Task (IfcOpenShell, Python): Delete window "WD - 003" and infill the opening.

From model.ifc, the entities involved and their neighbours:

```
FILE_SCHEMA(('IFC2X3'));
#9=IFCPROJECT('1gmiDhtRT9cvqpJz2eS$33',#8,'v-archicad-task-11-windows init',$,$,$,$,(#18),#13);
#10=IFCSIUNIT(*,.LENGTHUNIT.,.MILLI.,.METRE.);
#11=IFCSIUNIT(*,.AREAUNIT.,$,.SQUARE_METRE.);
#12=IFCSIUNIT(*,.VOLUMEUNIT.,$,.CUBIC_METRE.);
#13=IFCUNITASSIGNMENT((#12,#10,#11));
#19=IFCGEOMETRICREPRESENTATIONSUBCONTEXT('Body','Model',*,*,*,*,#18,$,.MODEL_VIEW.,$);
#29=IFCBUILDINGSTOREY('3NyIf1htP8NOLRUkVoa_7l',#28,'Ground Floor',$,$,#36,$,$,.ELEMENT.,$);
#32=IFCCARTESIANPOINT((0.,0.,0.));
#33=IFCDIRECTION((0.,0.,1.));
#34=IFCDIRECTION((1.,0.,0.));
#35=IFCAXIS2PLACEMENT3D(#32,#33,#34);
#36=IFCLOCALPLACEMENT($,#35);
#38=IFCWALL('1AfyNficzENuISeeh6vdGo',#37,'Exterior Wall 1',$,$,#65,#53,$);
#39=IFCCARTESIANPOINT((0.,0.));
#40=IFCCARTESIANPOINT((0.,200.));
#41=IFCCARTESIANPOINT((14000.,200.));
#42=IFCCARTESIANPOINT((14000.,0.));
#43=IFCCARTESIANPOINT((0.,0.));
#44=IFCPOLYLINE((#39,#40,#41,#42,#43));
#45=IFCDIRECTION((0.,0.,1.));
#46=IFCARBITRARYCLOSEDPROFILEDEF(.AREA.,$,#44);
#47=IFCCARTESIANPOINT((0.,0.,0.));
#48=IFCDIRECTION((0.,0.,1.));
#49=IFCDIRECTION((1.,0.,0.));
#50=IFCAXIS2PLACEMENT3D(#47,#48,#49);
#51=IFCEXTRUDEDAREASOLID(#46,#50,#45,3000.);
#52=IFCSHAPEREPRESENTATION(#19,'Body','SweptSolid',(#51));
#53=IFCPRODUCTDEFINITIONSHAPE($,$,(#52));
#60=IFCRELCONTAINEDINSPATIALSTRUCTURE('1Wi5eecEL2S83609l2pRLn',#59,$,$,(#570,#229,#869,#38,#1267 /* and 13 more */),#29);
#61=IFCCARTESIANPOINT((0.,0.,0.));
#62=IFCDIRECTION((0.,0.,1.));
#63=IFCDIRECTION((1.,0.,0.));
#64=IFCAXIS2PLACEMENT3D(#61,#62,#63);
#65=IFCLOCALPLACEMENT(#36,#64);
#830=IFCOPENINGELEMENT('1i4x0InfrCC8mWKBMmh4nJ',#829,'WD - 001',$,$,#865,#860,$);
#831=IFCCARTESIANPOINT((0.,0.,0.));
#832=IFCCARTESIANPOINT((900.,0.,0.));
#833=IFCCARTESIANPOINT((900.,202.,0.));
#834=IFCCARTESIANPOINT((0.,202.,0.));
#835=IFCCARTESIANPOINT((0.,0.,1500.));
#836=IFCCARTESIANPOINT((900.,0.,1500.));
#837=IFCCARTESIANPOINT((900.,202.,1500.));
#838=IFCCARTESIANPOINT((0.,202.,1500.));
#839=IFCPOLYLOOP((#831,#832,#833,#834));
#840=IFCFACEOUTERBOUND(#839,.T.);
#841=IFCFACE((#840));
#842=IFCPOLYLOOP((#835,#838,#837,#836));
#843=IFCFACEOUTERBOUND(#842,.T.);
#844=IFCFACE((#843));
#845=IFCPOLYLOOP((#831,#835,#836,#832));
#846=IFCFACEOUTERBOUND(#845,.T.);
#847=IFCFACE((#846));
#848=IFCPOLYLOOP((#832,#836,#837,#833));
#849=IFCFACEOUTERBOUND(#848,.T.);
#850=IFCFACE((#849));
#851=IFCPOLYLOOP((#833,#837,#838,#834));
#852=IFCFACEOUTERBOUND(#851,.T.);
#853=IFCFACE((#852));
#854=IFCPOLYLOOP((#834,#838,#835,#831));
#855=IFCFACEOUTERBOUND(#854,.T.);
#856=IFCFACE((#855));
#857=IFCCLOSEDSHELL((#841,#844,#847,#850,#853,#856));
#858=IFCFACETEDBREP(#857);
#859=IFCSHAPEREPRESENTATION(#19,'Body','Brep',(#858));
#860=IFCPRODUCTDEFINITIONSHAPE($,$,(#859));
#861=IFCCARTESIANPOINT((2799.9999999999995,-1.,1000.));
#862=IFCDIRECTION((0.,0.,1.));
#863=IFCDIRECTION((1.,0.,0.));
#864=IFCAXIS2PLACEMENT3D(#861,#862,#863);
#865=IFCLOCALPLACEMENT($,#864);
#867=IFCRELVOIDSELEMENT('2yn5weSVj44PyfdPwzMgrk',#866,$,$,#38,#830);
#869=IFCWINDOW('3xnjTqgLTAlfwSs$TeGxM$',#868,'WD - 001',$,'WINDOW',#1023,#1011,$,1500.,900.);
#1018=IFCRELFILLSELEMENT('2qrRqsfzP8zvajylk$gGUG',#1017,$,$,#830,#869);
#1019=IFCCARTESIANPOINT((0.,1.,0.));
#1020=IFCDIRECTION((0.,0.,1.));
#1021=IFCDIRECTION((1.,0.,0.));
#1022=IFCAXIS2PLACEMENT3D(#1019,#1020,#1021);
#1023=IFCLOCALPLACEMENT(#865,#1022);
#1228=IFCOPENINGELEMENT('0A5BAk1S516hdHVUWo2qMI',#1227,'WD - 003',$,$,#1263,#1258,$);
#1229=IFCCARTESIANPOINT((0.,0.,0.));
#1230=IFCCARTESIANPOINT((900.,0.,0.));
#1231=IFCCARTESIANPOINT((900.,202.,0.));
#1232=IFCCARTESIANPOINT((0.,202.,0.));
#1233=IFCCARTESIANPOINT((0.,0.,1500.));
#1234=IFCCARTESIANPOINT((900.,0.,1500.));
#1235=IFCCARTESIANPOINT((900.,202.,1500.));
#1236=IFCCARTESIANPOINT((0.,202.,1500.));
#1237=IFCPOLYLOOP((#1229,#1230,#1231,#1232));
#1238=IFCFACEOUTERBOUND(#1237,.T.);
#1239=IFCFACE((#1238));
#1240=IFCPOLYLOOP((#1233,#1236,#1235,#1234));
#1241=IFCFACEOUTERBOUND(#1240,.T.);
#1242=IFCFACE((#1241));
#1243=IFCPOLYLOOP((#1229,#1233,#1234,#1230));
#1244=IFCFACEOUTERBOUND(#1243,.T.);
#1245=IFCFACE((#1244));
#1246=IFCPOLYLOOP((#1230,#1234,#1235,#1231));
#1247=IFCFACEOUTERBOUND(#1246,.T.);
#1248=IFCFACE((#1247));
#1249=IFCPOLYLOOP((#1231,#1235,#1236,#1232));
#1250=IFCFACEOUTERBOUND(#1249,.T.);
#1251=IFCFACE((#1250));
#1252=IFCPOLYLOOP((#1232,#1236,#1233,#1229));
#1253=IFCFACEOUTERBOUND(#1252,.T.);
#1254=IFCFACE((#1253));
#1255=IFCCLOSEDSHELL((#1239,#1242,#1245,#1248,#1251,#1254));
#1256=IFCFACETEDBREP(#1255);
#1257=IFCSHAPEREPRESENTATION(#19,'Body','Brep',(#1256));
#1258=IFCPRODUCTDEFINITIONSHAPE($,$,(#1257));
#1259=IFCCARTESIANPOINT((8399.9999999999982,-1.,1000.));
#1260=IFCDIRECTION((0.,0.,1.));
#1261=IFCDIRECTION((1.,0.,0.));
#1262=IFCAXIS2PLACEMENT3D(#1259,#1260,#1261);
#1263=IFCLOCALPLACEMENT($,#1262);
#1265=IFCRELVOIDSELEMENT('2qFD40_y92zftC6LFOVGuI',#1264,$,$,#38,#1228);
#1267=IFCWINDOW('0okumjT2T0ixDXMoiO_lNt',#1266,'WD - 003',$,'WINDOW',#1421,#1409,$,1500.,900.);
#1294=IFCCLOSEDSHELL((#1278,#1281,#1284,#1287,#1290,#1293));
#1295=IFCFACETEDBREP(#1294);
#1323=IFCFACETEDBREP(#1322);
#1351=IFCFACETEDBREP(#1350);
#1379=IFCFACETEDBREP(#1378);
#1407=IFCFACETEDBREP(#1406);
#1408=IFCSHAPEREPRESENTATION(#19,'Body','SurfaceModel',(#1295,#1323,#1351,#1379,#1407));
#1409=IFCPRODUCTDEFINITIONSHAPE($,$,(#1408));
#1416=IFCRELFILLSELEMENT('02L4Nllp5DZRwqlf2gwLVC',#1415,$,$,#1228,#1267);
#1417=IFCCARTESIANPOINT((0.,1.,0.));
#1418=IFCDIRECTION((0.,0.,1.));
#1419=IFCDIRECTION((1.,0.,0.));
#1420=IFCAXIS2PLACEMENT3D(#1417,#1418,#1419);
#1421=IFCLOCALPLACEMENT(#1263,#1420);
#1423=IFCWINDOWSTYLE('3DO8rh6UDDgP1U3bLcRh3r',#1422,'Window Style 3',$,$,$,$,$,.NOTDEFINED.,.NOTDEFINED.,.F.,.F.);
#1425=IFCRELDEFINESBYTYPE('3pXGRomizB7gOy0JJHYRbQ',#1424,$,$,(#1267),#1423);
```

```python
import ifcopenshell
import ifcopenshell.api.feature
import ifcopenshell.api.root
import ifcopenshell.geom
import ifcopenshell.util.shape

model = ifcopenshell.open("model.ifc")
settings = ifcopenshell.geom.settings()


def volume(element):
    """Net volume in cubic metres, openings subtracted."""
    shape = ifcopenshell.geom.create_shape(settings, element)
    return ifcopenshell.util.shape.get_volume(shape.geometry)


window = model.by_id(1267)
opening = window.FillsVoids[0].RelatingOpeningElement
wall = opening.VoidsElements[0].RelatingBuildingElement
before = volume(wall)

ifcopenshell.api.root.remove_product(model, product=window)
ifcopenshell.api.feature.remove_feature(model, feature=opening)

after = volume(wall)

print(f"wall volume {before:.3f} -> {after:.3f} m3")

model.write("model_updated.ifc")
```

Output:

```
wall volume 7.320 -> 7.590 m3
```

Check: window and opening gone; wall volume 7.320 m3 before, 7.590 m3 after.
